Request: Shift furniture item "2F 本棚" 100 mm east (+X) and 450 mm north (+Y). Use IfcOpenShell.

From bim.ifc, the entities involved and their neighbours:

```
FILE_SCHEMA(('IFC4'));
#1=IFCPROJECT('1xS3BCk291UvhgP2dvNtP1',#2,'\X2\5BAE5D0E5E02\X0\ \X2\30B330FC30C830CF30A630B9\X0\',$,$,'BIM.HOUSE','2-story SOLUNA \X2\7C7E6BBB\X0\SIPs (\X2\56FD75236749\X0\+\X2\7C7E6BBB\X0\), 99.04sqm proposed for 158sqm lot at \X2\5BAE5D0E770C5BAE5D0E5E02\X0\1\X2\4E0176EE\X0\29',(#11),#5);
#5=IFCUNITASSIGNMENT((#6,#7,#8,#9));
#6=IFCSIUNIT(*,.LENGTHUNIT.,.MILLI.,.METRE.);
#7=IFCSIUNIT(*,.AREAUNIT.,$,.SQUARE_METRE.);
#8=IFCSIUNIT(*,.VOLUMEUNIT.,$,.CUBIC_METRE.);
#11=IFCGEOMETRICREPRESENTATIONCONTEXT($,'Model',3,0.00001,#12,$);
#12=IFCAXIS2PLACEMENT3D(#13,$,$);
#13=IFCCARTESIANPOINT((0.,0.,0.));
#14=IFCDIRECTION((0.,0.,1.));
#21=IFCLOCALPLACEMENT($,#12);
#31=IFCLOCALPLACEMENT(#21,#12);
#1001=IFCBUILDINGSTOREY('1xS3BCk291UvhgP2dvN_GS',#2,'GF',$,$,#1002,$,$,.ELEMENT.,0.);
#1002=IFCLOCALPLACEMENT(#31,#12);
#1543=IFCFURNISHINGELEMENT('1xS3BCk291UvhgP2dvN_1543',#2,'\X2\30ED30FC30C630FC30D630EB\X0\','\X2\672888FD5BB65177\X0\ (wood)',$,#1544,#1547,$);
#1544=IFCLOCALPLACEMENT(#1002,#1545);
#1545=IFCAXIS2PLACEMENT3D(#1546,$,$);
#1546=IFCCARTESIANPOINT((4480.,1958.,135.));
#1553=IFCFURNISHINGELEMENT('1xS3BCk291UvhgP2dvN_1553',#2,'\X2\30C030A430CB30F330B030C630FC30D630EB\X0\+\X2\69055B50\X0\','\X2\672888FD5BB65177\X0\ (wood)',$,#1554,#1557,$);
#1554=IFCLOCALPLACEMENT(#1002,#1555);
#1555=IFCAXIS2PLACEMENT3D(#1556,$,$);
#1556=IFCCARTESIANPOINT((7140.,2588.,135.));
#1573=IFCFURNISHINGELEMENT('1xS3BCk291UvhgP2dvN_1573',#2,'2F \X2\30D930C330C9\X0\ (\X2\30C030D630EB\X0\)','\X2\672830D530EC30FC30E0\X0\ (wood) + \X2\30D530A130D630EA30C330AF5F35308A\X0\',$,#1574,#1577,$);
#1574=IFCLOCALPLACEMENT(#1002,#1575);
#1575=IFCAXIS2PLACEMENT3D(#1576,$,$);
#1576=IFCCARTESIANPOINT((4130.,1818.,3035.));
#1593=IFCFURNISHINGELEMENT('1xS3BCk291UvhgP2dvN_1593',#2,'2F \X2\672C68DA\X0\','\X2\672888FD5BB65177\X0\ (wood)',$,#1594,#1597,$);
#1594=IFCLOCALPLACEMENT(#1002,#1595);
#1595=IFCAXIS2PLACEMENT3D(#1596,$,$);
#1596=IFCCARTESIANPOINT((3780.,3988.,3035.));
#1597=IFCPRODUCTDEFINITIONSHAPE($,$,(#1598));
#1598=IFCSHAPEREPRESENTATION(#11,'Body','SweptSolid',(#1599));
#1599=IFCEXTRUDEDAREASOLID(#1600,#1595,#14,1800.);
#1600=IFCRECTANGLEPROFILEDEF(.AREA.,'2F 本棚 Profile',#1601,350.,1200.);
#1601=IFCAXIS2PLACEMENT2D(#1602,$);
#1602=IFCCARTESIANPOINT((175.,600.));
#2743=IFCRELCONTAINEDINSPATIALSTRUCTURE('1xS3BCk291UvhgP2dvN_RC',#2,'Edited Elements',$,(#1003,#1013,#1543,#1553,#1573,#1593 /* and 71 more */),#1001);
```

```python
import ifcopenshell
import ifcopenshell.api.geometry
import ifcopenshell.util.placement

model = ifcopenshell.open("bim.ifc")

item = model.by_id(1593)
matrix = ifcopenshell.util.placement.get_local_placement(item.ObjectPlacement)
matrix[0, 3] += 100.0
matrix[1, 3] += 450.0
ifcopenshell.api.geometry.edit_object_placement(model, product=item, matrix=matrix, is_si=False)

print(ifcopenshell.util.placement.get_local_placement(item.ObjectPlacement).round(3) + 0.0)

model.write("bim-out.ifc")
```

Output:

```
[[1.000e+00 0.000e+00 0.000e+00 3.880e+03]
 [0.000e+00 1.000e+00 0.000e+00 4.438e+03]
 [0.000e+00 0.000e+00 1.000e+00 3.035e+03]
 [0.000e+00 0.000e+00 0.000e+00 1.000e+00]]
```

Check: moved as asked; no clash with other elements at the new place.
